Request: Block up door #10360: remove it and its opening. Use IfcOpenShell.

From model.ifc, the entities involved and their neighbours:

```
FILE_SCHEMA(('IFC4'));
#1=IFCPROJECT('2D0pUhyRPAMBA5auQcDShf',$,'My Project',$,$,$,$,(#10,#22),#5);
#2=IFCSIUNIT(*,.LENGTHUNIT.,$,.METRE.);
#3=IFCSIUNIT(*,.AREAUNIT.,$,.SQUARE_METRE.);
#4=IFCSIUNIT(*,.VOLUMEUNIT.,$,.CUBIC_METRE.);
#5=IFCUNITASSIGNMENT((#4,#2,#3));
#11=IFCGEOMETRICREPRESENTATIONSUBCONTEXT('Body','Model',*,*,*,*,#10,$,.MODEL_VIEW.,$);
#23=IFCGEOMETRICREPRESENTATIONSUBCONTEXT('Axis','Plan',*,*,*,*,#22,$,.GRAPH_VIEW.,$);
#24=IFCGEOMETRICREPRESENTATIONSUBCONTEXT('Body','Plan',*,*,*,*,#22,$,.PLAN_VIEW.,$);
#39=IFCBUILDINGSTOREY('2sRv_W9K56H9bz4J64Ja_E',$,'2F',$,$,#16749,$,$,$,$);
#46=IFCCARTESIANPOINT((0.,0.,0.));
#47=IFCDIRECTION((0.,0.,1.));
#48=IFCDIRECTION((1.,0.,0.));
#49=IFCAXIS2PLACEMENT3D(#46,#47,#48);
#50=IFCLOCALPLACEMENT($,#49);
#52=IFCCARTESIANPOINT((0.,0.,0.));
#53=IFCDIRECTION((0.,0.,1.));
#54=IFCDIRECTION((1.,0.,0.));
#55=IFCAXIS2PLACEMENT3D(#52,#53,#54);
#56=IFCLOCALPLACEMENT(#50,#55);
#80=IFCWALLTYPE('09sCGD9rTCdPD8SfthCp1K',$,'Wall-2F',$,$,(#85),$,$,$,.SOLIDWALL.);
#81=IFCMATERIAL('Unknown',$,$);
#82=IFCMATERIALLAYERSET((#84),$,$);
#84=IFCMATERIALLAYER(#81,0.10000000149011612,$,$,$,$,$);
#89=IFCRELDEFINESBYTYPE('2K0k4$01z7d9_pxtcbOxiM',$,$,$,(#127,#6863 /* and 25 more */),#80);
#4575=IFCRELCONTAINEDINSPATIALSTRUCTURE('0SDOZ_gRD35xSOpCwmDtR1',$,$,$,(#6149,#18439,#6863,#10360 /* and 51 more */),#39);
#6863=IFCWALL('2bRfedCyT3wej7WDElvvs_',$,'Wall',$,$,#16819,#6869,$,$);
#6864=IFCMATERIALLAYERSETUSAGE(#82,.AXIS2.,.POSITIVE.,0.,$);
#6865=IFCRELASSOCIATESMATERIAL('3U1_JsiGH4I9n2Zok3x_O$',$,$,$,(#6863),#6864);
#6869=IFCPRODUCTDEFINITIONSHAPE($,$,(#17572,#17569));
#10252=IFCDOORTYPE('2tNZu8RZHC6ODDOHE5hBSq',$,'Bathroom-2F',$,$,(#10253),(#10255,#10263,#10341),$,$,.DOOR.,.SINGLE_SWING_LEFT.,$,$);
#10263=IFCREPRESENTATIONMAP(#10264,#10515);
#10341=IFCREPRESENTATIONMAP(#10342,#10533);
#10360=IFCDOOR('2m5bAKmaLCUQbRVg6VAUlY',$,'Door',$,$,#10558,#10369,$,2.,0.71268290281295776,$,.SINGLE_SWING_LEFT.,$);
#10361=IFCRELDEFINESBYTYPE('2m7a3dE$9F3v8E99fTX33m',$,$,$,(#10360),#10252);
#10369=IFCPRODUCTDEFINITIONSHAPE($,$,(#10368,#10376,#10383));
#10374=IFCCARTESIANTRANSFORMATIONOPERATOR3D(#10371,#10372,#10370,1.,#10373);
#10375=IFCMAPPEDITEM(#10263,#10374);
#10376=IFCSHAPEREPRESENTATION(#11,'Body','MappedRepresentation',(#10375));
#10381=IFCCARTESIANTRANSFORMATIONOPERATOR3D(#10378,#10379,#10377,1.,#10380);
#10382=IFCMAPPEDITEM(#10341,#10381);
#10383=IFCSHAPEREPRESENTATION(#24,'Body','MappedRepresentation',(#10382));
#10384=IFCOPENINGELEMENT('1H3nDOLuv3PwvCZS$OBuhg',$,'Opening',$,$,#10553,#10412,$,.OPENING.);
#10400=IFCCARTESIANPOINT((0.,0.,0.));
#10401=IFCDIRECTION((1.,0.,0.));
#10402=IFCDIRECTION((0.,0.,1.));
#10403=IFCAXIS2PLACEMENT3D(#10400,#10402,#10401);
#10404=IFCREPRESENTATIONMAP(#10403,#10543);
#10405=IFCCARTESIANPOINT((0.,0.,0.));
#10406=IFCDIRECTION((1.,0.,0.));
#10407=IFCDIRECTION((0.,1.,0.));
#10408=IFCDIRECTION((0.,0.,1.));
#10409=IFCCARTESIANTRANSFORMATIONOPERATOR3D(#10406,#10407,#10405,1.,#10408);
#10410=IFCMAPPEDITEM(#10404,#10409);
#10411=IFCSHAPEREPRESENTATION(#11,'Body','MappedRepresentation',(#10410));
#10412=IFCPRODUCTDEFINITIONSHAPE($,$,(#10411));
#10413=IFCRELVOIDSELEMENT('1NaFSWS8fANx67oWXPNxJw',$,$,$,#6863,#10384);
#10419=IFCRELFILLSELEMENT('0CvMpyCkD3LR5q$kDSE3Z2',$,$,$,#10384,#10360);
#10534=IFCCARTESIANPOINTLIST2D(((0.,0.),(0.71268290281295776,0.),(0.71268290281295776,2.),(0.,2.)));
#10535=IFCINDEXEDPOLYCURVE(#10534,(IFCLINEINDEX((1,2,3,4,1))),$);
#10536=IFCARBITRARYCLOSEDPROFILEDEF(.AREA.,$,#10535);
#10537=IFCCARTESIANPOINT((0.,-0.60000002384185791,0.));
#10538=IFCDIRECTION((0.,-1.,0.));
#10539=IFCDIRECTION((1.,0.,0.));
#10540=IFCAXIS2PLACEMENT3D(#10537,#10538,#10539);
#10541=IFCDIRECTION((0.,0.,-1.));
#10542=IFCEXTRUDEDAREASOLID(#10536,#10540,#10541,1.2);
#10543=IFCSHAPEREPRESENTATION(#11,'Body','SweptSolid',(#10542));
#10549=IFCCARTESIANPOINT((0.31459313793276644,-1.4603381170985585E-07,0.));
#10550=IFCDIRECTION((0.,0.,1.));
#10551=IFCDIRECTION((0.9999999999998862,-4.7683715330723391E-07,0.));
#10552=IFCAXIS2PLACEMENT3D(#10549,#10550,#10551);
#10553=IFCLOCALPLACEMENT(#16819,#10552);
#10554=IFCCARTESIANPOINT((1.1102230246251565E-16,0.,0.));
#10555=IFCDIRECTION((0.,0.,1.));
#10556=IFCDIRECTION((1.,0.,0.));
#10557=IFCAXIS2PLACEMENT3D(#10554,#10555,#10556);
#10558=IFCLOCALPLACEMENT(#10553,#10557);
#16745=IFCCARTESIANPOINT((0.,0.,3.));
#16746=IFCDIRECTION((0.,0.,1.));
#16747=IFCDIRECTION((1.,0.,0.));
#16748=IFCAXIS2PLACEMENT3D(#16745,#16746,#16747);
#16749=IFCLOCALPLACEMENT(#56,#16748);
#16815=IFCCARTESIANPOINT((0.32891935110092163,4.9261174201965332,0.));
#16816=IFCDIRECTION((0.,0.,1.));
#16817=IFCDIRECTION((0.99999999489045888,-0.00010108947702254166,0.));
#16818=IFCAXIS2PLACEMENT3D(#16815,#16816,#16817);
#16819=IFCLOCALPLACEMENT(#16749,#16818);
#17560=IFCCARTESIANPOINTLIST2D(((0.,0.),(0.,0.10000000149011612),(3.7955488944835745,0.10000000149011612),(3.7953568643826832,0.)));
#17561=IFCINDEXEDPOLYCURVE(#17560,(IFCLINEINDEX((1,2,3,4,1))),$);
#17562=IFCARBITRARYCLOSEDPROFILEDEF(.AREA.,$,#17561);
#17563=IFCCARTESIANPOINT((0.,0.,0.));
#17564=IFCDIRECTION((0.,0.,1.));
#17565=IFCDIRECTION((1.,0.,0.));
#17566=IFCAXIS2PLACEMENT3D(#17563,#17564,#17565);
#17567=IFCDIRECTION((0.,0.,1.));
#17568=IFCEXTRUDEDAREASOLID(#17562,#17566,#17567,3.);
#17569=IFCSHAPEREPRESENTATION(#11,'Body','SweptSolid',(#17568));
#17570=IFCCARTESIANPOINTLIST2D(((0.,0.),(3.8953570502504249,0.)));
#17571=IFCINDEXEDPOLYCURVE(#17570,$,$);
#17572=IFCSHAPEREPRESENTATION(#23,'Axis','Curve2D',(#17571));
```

```python
import ifcopenshell
import ifcopenshell.api.feature
import ifcopenshell.api.root
import ifcopenshell.geom
import ifcopenshell.util.shape

model = ifcopenshell.open("model.ifc")
settings = ifcopenshell.geom.settings()


def volume(element):
    """Net volume in cubic metres, openings subtracted."""
    shape = ifcopenshell.geom.create_shape(settings, element)
    return ifcopenshell.util.shape.get_volume(shape.geometry)


door = model.by_guid("2m5bAKmaLCUQbRVg6VAUlY")
opening = door.FillsVoids[0].RelatingOpeningElement
wall = opening.VoidsElements[0].RelatingBuildingElement
before = volume(wall)

ifcopenshell.api.root.remove_product(model, product=door)
ifcopenshell.api.feature.remove_feature(model, feature=opening)

after = volume(wall)

print(f"wall volume {before:.3f} -> {after:.3f} m3")

model.write("model_updated.ifc")
```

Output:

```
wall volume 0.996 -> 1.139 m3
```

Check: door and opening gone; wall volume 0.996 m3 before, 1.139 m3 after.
